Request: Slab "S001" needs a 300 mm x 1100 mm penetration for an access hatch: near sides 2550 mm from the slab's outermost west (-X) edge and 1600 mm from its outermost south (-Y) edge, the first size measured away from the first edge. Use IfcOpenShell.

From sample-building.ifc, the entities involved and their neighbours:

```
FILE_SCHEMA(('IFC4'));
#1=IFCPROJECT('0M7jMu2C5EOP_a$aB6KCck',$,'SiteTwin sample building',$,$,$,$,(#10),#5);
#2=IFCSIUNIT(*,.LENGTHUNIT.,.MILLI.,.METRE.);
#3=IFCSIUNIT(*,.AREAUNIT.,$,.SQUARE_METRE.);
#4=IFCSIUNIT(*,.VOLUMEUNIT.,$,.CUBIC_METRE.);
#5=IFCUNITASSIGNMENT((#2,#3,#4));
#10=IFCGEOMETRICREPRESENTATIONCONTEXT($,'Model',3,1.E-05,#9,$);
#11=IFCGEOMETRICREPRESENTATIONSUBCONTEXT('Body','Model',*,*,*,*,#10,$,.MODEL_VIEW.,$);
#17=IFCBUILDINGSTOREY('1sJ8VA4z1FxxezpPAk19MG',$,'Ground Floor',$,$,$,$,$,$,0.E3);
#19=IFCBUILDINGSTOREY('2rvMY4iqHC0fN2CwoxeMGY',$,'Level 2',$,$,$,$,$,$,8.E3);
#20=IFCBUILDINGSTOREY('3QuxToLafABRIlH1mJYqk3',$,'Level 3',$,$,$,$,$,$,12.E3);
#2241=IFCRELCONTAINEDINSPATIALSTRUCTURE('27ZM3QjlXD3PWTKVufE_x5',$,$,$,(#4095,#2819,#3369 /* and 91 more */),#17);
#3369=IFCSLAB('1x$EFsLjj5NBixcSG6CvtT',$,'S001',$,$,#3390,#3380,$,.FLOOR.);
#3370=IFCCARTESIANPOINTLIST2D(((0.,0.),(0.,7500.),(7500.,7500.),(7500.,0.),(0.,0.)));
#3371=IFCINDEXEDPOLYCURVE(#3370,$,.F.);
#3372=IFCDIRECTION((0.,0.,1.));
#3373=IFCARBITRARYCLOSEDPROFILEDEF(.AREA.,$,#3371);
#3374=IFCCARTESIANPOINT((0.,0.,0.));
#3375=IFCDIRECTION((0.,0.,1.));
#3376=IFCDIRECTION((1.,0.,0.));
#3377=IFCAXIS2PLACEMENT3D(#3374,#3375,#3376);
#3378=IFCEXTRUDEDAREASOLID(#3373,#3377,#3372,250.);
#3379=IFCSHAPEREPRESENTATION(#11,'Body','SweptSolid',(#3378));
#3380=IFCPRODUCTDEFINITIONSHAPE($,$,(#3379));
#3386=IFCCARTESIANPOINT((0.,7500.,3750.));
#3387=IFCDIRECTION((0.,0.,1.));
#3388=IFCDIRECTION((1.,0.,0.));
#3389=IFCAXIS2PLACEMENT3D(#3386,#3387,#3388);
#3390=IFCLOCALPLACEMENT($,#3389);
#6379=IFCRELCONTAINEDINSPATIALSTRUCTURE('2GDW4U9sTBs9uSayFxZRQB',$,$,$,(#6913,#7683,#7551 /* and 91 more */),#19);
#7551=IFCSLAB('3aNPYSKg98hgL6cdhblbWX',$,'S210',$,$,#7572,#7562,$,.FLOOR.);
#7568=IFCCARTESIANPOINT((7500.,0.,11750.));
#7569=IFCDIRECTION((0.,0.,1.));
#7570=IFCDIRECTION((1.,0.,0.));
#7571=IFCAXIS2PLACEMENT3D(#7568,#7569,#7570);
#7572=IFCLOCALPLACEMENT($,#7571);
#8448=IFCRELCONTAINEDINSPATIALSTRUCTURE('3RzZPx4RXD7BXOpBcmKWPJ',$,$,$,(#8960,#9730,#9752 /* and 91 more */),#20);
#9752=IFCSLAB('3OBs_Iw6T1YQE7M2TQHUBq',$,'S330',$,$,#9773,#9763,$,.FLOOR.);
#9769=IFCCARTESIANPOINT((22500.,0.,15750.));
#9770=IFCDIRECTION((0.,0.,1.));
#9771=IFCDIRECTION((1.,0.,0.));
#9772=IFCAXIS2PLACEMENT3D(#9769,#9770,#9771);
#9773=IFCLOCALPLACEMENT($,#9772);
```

```python
import numpy as np
import ifcopenshell
import ifcopenshell.api.feature
import ifcopenshell.api.geometry
import ifcopenshell.api.root
import ifcopenshell.geom
import ifcopenshell.util.placement
import ifcopenshell.util.representation
import ifcopenshell.util.shape
import ifcopenshell.util.unit

model = ifcopenshell.open("sample-building.ifc")
unit_scale = ifcopenshell.util.unit.calculate_unit_scale(model)
settings = ifcopenshell.geom.settings()


def volume(element):
    """Net volume in cubic metres, openings subtracted."""
    shape = ifcopenshell.geom.create_shape(settings, element)
    return ifcopenshell.util.shape.get_volume(shape.geometry)


slab = model.by_guid("1x$EFsLjj5NBixcSG6CvtT")
before = volume(slab)

# Extent in the slab's own axes, in metres. The edges named are its -X and -Y sides.
slab_shape = ifcopenshell.geom.create_shape(settings, slab)
vertices = ifcopenshell.util.shape.get_vertices(slab_shape.geometry)
x_min, y_min, bottom = vertices.min(axis=0)
top = vertices[:, 2].max()

opening = ifcopenshell.api.root.create_entity(model, ifc_class="IfcOpeningElement", name="Access hatch opening", predefined_type="OPENING")
context = ifcopenshell.util.representation.get_context(model, "Model", "Body", "MODEL_VIEW")
width, depth = 0.3, 1.1
outline = [(0.0, 0.0), (width, 0.0), (width, depth), (0.0, depth), (0.0, 0.0)]
# Overshoot both faces by 50 mm so the cut is clean.
shape = ifcopenshell.api.geometry.add_slab_representation(
    model, context=context, depth=top - bottom + 0.1, polyline=outline
)
ifcopenshell.api.geometry.assign_representation(model, product=opening, representation=shape)

matrix = ifcopenshell.util.placement.get_local_placement(slab.ObjectPlacement)
matrix[:, 3] = matrix @ np.append(np.array([x_min + 2.55, y_min + 1.6, bottom - 0.05]) / unit_scale, 1.0)
ifcopenshell.api.geometry.edit_object_placement(model, product=opening, matrix=matrix, is_si=False)
ifcopenshell.api.feature.add_feature(model, feature=opening, element=slab)

after = volume(slab)

print(f"slab volume {before:.3f} -> {after:.3f} m3")

model.write("sample-building_v2.ifc")
```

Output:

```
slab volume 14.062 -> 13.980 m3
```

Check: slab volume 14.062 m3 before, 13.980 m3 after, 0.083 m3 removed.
